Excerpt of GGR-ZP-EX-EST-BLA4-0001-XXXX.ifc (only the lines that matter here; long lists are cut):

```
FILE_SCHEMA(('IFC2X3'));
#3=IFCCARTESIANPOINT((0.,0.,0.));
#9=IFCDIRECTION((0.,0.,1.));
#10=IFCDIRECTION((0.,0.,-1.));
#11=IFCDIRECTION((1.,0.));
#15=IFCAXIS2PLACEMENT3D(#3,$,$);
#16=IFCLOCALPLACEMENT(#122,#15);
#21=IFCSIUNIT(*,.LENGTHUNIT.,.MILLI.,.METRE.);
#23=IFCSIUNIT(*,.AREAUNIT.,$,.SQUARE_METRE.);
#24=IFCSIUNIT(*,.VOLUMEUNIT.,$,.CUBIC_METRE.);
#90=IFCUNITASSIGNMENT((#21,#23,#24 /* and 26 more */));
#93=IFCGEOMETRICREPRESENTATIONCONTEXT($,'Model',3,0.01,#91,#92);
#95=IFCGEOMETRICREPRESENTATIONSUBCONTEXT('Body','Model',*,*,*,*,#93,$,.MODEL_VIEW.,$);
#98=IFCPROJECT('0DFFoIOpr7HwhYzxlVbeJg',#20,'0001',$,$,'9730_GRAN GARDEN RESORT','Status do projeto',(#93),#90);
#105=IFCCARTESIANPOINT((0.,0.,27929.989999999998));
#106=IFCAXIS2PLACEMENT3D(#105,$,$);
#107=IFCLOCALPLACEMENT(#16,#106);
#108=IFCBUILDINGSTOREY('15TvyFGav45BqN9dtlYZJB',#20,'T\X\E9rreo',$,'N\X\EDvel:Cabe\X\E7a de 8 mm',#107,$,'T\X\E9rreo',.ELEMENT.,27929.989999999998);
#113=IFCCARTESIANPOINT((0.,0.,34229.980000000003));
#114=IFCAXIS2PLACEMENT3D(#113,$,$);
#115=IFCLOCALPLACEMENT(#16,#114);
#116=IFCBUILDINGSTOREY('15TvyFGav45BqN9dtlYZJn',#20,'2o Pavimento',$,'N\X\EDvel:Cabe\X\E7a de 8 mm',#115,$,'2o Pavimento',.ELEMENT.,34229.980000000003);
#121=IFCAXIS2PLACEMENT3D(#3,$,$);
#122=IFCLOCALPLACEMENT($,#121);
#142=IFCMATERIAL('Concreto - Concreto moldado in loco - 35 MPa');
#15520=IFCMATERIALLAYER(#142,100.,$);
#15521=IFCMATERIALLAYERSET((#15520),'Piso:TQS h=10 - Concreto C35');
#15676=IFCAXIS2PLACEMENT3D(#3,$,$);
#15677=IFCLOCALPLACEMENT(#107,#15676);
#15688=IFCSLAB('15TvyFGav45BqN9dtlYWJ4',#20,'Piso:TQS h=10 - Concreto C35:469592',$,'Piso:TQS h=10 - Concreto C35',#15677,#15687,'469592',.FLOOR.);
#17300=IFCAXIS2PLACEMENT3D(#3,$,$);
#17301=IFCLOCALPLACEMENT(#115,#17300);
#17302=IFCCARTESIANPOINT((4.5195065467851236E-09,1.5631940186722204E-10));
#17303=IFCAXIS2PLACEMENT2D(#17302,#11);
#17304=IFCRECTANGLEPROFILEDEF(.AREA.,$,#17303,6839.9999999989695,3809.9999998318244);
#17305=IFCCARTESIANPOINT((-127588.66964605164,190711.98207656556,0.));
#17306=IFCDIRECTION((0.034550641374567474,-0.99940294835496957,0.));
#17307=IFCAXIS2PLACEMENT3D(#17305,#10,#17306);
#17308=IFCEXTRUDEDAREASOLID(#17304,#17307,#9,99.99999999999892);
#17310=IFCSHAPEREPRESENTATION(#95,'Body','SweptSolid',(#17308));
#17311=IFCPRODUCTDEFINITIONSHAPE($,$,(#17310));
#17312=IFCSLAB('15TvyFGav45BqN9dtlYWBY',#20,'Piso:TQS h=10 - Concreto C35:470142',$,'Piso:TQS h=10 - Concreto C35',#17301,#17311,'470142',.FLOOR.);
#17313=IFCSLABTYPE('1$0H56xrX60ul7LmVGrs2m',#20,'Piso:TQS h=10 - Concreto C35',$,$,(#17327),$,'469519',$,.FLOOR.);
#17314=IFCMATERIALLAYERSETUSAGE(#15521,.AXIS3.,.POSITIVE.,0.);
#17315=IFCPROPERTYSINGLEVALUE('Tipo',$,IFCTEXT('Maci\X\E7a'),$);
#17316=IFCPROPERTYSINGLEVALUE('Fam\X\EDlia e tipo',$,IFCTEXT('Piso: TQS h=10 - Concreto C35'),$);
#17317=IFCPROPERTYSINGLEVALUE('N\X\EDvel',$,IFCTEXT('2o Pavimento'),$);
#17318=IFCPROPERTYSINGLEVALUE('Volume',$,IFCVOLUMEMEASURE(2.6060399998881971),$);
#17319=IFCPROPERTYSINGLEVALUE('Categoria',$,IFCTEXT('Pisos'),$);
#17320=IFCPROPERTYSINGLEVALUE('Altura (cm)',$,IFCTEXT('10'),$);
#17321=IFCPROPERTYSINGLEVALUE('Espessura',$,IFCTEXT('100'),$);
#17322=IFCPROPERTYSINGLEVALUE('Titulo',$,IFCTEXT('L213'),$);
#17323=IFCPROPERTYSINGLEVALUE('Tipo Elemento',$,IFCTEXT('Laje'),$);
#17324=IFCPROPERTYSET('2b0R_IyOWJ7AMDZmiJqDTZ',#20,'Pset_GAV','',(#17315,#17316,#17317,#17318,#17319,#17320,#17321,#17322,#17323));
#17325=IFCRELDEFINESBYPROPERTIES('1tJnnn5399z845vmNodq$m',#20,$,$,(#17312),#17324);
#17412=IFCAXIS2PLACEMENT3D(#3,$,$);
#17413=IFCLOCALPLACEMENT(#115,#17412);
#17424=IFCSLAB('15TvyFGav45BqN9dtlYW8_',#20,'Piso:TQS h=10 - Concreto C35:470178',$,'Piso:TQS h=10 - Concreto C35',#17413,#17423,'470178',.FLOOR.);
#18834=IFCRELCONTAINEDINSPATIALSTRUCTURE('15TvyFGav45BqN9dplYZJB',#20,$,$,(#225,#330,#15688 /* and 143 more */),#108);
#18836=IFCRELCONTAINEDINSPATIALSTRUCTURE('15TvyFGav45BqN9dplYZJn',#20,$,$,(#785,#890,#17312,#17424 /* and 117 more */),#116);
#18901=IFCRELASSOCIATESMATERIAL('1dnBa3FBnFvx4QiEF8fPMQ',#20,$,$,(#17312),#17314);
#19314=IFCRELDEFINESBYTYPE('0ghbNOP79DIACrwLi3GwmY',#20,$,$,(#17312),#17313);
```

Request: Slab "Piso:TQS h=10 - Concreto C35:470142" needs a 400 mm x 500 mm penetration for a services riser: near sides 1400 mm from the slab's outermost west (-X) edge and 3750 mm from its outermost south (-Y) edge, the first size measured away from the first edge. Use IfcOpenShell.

```python
import numpy as np
import ifcopenshell
import ifcopenshell.api.feature
import ifcopenshell.api.geometry
import ifcopenshell.api.pset
import ifcopenshell.api.root
import ifcopenshell.geom
import ifcopenshell.util.element
import ifcopenshell.util.placement
import ifcopenshell.util.representation
import ifcopenshell.util.shape
import ifcopenshell.util.unit

model = ifcopenshell.open("GGR-ZP-EX-EST-BLA4-0001-XXXX.ifc")
unit_scale = ifcopenshell.util.unit.calculate_unit_scale(model)
volume_scale = ifcopenshell.util.unit.calculate_unit_scale(model, "VOLUMEUNIT")
settings = ifcopenshell.geom.settings()


def volume(element):
    """Net volume in cubic metres, openings subtracted."""
    shape = ifcopenshell.geom.create_shape(settings, element)
    return ifcopenshell.util.shape.get_volume(shape.geometry)


slab = model.by_guid("15TvyFGav45BqN9dtlYWBY")
before = volume(slab)

# Extent in the slab's own axes, in metres. The edges named are its -X and -Y sides.
slab_shape = ifcopenshell.geom.create_shape(settings, slab)
vertices = ifcopenshell.util.shape.get_vertices(slab_shape.geometry)
x_min, y_min, bottom = vertices.min(axis=0)
top = vertices[:, 2].max()

opening = ifcopenshell.api.root.create_entity(model, ifc_class="IfcOpeningElement", name="Services riser opening")
context = ifcopenshell.util.representation.get_context(model, "Model", "Body", "MODEL_VIEW")
width, depth = 0.4, 0.5
outline = [(0.0, 0.0), (width, 0.0), (width, depth), (0.0, depth), (0.0, 0.0)]
# Overshoot both faces by 50 mm so the cut is clean.
shape = ifcopenshell.api.geometry.add_slab_representation(
    model, context=context, depth=top - bottom + 0.1, polyline=outline
)
ifcopenshell.api.geometry.assign_representation(model, product=opening, representation=shape)

matrix = ifcopenshell.util.placement.get_local_placement(slab.ObjectPlacement)
matrix[:, 3] = matrix @ np.append(np.array([x_min + 1.4, y_min + 3.75, bottom - 0.05]) / unit_scale, 1.0)
ifcopenshell.api.geometry.edit_object_placement(model, product=opening, matrix=matrix, is_si=False)
ifcopenshell.api.feature.add_feature(model, feature=opening, element=slab)

after = volume(slab)

# Update the slab's stored quantities.
pset = model.by_id(ifcopenshell.util.element.get_pset(slab, "Pset_GAV", should_inherit=False)["id"])
ifcopenshell.api.pset.edit_pset(model, pset=pset, properties={
    "Volume": model.create_entity("IfcVolumeMeasure", after / volume_scale),
})

print(f"slab volume {before:.3f} -> {after:.3f} m3")

model.write("GGR-ZP-EX-EST-BLA4-0001-XXXX_rev.ifc")
```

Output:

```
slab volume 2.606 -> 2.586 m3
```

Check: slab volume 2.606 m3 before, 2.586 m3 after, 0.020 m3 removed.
